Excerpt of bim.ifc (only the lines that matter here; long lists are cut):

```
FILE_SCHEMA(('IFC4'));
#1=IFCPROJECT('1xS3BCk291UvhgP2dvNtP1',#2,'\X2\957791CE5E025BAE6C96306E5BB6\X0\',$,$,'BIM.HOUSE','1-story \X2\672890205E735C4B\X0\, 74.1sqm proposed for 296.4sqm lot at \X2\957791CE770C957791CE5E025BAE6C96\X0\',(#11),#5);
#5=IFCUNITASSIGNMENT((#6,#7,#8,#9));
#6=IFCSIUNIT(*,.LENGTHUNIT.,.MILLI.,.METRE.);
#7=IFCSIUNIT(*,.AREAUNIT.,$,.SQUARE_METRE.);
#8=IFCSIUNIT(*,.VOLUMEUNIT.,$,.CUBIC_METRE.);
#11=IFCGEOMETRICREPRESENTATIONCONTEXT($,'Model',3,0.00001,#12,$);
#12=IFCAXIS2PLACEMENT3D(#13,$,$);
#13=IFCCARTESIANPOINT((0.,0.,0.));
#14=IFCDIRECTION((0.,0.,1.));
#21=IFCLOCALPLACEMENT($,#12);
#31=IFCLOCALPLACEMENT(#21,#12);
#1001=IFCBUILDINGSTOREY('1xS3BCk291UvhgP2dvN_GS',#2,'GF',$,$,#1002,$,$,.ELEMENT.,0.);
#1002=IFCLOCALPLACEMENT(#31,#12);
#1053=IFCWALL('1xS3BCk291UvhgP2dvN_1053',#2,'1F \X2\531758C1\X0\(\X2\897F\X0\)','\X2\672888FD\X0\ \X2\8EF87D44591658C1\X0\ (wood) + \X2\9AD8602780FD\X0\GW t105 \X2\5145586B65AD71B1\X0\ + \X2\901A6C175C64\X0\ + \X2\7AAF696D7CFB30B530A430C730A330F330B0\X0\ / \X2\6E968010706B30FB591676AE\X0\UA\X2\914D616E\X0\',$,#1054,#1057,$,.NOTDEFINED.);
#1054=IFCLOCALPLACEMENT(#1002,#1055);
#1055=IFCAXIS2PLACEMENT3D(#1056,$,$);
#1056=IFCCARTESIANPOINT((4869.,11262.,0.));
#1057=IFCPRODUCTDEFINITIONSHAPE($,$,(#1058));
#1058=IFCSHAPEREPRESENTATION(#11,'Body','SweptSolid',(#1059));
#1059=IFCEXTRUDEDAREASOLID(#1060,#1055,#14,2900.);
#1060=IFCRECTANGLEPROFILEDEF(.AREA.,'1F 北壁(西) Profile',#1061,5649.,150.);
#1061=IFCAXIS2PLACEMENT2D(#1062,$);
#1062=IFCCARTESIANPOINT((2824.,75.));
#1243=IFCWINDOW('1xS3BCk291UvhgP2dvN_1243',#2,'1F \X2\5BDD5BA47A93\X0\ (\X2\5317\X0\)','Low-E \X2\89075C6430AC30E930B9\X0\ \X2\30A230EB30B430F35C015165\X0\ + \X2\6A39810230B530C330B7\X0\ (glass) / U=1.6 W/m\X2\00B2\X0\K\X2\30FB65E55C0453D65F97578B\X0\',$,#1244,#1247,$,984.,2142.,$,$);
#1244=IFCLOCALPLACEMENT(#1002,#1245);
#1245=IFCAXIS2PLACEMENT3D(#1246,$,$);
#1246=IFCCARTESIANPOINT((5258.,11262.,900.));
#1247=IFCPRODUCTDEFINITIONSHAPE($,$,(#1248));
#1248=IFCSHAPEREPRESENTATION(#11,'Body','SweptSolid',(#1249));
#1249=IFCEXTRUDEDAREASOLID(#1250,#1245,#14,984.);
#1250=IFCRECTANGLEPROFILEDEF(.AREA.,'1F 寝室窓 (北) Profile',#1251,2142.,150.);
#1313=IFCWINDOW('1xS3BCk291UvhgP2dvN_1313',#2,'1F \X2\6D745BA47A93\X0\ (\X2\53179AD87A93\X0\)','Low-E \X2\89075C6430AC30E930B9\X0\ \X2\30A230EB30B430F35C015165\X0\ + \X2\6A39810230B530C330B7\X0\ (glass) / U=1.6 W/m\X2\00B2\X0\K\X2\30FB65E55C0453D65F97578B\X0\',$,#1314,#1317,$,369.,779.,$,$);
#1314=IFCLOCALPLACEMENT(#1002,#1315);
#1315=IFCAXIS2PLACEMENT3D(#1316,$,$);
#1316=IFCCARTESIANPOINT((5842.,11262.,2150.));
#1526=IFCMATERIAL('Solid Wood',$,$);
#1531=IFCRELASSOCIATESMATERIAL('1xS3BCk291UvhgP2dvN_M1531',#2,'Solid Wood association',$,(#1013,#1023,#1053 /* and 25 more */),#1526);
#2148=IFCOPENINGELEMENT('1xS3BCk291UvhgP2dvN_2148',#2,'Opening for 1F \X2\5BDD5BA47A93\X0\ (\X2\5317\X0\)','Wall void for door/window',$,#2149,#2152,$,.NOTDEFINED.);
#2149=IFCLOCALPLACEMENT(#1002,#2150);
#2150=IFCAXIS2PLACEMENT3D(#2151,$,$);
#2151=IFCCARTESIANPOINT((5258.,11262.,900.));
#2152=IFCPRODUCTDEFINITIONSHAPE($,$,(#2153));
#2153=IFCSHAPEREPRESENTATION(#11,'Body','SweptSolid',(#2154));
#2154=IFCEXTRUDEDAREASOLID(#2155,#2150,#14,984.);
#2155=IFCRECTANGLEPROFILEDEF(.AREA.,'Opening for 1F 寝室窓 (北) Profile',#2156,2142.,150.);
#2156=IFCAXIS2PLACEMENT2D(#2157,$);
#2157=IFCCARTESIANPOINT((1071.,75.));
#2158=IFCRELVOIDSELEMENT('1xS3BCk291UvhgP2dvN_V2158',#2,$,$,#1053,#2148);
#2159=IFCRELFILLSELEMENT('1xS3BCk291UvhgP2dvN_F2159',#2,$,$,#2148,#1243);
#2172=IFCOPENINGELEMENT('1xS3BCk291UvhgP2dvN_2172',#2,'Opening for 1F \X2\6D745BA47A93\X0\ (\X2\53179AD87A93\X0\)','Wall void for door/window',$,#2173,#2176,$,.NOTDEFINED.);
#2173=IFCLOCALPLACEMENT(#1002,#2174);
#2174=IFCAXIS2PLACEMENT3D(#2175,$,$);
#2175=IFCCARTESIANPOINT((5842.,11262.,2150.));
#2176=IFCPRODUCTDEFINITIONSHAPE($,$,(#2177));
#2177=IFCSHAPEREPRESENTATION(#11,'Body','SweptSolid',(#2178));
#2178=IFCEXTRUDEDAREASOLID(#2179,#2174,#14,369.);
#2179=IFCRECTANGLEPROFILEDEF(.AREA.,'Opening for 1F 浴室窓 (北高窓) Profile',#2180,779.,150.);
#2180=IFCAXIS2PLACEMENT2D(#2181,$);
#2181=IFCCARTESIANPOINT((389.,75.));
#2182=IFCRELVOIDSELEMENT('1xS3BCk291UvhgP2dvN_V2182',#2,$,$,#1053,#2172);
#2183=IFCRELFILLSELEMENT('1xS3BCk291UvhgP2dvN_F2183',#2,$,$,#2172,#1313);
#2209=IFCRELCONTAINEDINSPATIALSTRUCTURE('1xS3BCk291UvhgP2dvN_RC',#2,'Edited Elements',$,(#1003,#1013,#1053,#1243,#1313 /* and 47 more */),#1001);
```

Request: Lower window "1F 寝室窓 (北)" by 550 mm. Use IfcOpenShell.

```python
import numpy as np
import ifcopenshell
import ifcopenshell.api.geometry
import ifcopenshell.util.placement
import ifcopenshell.util.unit

model = ifcopenshell.open("bim.ifc")
unit_scale = ifcopenshell.util.unit.calculate_unit_scale(model)

window = model.by_guid("1xS3BCk291UvhgP2dvN_1243")
opening = window.FillsVoids[0].RelatingOpeningElement
dz = -0.55 / unit_scale

shift = np.array([0.0, 0.0, dz])
# The window is not placed relative to its opening, so move both.
for product in (opening, window):
    matrix = ifcopenshell.util.placement.get_local_placement(product.ObjectPlacement)
    matrix[:3, 3] += shift
    ifcopenshell.api.geometry.edit_object_placement(model, product=product, matrix=matrix, is_si=False)

print(f"moved by {dz * unit_scale:+.3f} m")

model.write("bim_updated.ifc")
```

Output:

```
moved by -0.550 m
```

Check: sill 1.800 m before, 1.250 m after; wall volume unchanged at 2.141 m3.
